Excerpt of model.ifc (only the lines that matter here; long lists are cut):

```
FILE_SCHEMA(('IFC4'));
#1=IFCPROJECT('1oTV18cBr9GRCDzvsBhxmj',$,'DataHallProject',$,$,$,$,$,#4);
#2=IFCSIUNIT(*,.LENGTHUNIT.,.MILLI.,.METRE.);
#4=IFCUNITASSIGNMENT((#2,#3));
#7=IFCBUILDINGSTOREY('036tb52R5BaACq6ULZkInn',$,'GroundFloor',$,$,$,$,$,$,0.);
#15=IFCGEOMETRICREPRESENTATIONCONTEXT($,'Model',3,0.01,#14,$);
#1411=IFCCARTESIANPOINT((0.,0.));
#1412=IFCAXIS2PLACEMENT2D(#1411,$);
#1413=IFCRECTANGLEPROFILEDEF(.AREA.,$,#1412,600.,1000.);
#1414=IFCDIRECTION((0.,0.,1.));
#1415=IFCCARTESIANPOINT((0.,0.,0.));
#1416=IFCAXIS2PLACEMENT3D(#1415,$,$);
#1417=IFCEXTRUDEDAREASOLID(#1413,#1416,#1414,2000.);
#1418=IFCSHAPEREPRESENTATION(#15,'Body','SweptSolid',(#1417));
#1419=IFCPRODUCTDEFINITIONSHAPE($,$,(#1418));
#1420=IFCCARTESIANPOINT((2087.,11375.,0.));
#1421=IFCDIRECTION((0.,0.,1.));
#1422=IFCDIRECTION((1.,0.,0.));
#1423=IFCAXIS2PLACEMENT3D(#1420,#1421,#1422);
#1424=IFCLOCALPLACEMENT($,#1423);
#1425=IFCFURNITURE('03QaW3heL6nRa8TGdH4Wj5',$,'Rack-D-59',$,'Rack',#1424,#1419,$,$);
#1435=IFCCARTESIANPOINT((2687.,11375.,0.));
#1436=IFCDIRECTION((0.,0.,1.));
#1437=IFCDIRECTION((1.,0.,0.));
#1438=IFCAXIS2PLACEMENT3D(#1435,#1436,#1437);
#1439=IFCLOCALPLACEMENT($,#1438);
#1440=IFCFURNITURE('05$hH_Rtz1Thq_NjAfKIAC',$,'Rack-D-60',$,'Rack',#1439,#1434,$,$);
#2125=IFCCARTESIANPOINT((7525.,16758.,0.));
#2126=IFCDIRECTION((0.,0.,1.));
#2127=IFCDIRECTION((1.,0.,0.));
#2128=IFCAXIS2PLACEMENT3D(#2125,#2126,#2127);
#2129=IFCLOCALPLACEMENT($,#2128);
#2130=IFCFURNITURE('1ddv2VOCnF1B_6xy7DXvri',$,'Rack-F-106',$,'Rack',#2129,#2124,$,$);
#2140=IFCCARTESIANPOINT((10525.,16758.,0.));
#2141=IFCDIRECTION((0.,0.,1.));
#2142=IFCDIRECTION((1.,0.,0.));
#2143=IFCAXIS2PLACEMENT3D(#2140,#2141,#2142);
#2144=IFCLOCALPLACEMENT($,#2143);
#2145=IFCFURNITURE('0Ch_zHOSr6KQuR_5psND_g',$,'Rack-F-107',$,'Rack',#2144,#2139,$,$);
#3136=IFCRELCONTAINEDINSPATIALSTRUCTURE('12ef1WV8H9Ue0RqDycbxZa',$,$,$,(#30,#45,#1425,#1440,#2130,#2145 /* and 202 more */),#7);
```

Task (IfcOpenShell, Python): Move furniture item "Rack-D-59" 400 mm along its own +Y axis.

```python
import ifcopenshell
import ifcopenshell.api.geometry
import ifcopenshell.util.placement
import ifcopenshell.util.unit

model = ifcopenshell.open("model.ifc")
unit_scale = ifcopenshell.util.unit.calculate_unit_scale(model)

item = model.by_id(1425)
matrix = ifcopenshell.util.placement.get_local_placement(item.ObjectPlacement)
matrix[:3, 3] += matrix[:3, 1] * 0.4 / unit_scale
ifcopenshell.api.geometry.edit_object_placement(model, product=item, matrix=matrix, is_si=False)

print(ifcopenshell.util.placement.get_local_placement(item.ObjectPlacement).round(3) + 0.0)

model.write("model_edited.ifc")
```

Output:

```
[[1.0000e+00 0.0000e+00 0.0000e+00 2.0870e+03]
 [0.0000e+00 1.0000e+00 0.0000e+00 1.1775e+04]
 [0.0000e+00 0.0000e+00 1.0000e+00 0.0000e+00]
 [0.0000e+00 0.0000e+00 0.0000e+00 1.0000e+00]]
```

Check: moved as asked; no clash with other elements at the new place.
